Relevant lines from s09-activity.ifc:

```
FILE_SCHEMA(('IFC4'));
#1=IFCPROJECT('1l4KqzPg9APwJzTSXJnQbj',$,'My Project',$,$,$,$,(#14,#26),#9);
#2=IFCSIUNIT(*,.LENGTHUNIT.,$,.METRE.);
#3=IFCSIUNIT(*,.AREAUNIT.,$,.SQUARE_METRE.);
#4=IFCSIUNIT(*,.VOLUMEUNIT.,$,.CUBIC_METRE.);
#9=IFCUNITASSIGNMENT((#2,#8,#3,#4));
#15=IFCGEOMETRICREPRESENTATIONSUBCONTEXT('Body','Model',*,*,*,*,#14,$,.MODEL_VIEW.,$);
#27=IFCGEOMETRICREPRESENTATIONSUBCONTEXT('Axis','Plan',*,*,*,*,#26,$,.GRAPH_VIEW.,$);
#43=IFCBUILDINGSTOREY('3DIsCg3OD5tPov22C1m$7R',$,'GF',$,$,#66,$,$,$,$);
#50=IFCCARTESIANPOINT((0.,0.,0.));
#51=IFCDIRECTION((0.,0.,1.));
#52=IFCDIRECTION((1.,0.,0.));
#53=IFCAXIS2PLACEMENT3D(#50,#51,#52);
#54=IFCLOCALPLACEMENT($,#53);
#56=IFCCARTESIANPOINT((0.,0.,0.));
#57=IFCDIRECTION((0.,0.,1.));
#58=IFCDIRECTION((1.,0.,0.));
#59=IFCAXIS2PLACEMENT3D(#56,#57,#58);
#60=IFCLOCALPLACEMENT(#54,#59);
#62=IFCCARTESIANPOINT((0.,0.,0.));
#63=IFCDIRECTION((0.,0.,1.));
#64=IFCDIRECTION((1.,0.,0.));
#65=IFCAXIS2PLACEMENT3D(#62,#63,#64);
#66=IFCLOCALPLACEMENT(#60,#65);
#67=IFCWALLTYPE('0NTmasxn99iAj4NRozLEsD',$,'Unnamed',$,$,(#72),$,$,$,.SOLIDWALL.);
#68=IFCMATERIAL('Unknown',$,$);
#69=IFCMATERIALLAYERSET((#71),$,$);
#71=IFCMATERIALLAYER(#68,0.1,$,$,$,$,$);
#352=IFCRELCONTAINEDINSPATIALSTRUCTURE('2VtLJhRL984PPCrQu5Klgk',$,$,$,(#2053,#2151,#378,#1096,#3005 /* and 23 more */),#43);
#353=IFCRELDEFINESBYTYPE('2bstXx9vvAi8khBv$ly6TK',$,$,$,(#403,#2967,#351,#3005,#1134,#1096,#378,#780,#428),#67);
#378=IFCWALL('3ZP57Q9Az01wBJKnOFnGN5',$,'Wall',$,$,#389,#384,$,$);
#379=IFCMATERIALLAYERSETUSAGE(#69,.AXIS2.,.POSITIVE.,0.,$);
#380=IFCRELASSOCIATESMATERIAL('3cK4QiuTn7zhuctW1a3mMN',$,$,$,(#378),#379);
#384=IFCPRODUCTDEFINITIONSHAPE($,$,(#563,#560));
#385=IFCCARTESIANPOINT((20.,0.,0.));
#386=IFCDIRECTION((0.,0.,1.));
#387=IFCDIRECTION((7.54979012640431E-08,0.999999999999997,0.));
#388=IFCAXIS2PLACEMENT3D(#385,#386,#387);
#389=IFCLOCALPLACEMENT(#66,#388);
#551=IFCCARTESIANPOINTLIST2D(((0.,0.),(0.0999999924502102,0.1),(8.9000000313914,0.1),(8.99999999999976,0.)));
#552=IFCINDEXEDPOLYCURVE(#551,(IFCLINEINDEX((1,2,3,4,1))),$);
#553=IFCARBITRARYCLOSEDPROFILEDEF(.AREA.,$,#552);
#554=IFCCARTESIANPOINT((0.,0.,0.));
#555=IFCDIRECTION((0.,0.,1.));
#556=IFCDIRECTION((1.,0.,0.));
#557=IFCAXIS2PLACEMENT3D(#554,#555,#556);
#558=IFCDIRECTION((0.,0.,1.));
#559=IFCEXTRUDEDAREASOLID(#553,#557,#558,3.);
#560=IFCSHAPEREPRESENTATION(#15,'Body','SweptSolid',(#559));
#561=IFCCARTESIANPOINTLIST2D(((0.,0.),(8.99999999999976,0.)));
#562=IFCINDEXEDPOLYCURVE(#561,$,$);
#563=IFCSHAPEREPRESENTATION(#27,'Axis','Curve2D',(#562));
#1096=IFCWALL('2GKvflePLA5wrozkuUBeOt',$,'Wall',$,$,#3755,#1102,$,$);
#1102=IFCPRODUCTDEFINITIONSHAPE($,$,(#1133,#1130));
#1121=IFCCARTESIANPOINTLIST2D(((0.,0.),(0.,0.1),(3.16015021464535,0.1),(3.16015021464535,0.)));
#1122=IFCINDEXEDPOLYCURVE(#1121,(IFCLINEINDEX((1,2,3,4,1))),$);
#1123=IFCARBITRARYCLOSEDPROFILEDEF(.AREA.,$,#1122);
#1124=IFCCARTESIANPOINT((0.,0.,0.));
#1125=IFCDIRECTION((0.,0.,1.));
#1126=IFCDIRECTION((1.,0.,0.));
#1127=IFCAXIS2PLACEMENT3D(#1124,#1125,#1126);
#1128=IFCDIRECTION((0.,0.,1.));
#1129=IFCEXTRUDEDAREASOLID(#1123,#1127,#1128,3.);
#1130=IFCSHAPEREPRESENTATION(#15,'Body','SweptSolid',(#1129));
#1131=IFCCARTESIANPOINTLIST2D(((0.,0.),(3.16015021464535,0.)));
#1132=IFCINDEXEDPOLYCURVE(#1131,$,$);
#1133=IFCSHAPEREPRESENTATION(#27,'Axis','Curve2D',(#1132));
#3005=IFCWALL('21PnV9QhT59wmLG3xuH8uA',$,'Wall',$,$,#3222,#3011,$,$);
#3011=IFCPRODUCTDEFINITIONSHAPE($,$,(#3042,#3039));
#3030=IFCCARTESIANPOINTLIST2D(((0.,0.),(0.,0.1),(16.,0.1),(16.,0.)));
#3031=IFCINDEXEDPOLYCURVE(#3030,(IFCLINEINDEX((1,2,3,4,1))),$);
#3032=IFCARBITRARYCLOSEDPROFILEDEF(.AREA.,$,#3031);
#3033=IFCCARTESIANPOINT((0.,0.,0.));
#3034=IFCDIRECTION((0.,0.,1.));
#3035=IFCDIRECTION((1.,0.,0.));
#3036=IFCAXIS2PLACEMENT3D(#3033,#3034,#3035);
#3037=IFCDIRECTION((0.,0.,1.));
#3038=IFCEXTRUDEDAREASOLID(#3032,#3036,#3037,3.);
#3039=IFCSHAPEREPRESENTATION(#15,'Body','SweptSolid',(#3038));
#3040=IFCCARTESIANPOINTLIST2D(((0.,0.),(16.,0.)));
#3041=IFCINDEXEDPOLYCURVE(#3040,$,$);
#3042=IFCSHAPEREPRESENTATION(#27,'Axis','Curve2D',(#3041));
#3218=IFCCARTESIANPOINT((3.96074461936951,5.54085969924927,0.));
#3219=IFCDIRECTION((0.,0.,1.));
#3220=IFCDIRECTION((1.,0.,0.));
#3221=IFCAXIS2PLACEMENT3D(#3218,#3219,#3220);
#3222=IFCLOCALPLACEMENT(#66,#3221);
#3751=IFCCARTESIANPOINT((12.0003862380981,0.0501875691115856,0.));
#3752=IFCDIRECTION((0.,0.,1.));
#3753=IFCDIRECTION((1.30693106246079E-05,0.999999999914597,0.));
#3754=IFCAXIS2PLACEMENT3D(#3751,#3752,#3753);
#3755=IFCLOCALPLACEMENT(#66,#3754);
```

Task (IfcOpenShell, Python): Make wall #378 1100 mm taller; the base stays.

```python
import ifcopenshell
import ifcopenshell.geom
import ifcopenshell.util.representation
import ifcopenshell.util.shape
import ifcopenshell.util.unit

model = ifcopenshell.open("s09-activity.ifc")
unit_scale = ifcopenshell.util.unit.calculate_unit_scale(model)
settings = ifcopenshell.geom.settings()


def volume(element):
    """Net volume in cubic metres, openings subtracted."""
    shape = ifcopenshell.geom.create_shape(settings, element)
    return ifcopenshell.util.shape.get_volume(shape.geometry)


wall = model.by_guid("3ZP57Q9Az01wBJKnOFnGN5")
before = volume(wall)

body = ifcopenshell.util.representation.get_representation(wall, "Model", "Body")
solid = body.Items[0]
old_height = solid.Depth
solid.Depth += 1.1 / unit_scale
after = volume(wall)

print(f"height {old_height:g} -> {solid.Depth:g}, volume {before:.3f} -> {after:.3f} m3")

model.write("s09-activity_v2.ifc")
```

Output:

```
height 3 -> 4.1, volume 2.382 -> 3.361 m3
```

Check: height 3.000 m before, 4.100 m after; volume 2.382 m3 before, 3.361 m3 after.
